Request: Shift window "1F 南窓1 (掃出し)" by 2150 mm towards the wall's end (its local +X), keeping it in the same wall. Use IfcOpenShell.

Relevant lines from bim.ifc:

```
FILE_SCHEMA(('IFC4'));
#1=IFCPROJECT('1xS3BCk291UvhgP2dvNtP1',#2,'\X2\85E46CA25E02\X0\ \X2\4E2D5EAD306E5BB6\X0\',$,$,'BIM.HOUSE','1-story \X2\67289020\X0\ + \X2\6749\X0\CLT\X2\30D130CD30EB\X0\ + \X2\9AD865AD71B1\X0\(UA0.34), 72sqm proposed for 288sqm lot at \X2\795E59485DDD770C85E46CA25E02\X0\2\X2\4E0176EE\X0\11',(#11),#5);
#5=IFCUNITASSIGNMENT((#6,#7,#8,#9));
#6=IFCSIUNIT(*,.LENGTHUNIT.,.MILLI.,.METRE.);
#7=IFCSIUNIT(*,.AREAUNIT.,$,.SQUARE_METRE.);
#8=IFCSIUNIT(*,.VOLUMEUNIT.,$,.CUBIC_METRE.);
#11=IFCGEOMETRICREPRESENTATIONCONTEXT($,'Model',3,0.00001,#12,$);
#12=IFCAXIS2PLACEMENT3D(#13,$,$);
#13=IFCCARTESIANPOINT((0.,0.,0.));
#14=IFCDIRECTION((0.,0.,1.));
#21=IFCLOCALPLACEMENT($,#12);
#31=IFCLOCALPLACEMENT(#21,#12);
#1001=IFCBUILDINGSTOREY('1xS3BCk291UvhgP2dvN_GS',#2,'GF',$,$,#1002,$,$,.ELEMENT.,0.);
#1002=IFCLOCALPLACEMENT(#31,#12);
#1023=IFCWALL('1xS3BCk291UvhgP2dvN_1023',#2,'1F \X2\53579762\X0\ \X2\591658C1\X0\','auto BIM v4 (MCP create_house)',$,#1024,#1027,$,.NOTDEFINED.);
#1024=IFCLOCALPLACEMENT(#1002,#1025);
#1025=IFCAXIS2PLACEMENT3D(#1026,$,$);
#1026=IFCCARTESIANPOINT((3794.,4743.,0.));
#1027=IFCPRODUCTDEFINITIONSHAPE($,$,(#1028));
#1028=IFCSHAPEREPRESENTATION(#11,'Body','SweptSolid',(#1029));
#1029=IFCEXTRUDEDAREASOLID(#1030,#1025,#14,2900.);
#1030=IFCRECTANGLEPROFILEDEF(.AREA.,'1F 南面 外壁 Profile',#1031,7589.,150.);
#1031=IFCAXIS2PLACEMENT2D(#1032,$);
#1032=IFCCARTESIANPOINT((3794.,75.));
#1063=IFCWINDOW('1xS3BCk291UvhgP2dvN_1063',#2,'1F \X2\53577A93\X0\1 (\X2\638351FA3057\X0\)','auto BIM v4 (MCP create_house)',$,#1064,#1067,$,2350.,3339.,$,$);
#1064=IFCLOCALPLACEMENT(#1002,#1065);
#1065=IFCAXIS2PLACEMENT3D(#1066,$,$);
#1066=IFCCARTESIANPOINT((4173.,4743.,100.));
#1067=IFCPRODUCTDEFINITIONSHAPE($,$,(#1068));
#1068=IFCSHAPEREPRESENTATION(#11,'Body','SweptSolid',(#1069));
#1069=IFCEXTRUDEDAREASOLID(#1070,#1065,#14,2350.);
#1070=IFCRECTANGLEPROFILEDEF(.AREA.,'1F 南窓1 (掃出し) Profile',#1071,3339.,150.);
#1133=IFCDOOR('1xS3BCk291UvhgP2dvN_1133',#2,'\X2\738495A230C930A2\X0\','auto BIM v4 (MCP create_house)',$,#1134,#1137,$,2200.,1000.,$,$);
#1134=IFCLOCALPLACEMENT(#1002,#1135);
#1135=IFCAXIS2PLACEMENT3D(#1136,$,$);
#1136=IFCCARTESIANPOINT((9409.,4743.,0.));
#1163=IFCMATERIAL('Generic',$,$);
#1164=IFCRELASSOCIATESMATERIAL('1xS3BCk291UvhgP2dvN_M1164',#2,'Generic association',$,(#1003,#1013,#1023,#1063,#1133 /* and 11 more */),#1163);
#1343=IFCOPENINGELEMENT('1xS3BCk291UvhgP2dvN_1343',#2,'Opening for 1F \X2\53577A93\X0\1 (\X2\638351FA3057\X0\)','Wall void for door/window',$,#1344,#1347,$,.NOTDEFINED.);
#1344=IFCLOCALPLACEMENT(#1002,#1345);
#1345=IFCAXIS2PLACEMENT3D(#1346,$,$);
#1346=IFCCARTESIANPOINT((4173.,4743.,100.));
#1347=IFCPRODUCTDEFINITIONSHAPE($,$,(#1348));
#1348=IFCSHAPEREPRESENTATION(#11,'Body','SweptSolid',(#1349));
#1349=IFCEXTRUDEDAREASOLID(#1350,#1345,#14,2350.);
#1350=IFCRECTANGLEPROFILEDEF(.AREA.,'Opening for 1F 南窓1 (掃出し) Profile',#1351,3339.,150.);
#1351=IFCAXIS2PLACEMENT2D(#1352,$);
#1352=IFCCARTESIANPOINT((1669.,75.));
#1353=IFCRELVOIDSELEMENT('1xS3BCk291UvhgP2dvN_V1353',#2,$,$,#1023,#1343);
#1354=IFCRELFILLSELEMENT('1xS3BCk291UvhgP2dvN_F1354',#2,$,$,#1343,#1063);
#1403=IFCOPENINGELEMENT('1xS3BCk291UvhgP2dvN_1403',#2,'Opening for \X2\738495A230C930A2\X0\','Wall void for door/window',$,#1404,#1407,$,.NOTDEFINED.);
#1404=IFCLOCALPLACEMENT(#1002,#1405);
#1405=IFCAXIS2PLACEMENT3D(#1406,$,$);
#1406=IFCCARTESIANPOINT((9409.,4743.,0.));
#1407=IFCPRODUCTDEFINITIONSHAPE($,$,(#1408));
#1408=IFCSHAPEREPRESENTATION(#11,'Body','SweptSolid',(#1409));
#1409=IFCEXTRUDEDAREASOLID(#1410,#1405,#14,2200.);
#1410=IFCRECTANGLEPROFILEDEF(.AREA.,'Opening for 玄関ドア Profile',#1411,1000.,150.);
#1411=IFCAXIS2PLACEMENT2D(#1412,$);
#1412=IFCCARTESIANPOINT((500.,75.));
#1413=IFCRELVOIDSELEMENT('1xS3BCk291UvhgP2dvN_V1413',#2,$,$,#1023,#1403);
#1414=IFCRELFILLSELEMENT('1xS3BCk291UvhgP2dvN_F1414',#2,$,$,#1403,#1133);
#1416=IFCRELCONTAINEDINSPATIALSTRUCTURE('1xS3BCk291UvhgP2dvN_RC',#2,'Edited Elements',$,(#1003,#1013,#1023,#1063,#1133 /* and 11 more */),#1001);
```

```python
import ifcopenshell
import ifcopenshell.api.geometry
import ifcopenshell.util.placement

model = ifcopenshell.open("bim.ifc")

window = model.by_guid("1xS3BCk291UvhgP2dvN_1063")
opening = window.FillsVoids[0].RelatingOpeningElement
wall = opening.VoidsElements[0].RelatingBuildingElement

wall_matrix = ifcopenshell.util.placement.get_local_placement(wall.ObjectPlacement)
shift = wall_matrix[:3, 0] * 2150.0
before = ifcopenshell.util.placement.get_local_placement(window.ObjectPlacement)[:3, 3].copy()

# The window is not placed relative to its opening, so move both.
for product in (opening, window):
    matrix = ifcopenshell.util.placement.get_local_placement(product.ObjectPlacement)
    matrix[:3, 3] += shift
    ifcopenshell.api.geometry.edit_object_placement(model, product=product, matrix=matrix, is_si=False)

after = ifcopenshell.util.placement.get_local_placement(window.ObjectPlacement)[:3, 3]
print("window moved by", (after - before).round(3) + 0.0)

model.write("bim_updated.ifc")
```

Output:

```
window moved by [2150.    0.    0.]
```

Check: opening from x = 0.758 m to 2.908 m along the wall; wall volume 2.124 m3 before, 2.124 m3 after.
